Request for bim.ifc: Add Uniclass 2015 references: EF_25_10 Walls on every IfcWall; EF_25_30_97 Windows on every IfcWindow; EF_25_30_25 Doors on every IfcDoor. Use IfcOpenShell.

First a look at what the model holds.

```python
import ifcopenshell

model = ifcopenshell.open("bim.ifc")
print(model.schema)
print("classifications:", [c.Name for c in model.by_type("IfcClassification")])
for ifc_class in ("IfcDoor", "IfcRoof", "IfcStair", "IfcWall", "IfcWindow"):
    print(ifc_class, len(model.by_type(ifc_class)))
```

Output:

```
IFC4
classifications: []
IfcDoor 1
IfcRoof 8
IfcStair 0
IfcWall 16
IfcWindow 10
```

```python
import ifcopenshell
import ifcopenshell.api.classification

model = ifcopenshell.open("bim.ifc")

system = ifcopenshell.api.classification.add_classification(model, classification="Uniclass 2015")

codes = {
    "IfcWall": ("EF_25_10", "Walls"),
    "IfcWindow": ("EF_25_30_97", "Windows"),
    "IfcDoor": ("EF_25_30_25", "Doors"),
}
for ifc_class, (code, name) in codes.items():
    products = model.by_type(ifc_class)
    ifcopenshell.api.classification.add_reference(
        model, products=products, classification=system, identification=code, name=name
    )
    print(code, len(products))

model.write("bim-out.ifc")
```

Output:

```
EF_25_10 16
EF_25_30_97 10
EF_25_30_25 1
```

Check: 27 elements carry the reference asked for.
